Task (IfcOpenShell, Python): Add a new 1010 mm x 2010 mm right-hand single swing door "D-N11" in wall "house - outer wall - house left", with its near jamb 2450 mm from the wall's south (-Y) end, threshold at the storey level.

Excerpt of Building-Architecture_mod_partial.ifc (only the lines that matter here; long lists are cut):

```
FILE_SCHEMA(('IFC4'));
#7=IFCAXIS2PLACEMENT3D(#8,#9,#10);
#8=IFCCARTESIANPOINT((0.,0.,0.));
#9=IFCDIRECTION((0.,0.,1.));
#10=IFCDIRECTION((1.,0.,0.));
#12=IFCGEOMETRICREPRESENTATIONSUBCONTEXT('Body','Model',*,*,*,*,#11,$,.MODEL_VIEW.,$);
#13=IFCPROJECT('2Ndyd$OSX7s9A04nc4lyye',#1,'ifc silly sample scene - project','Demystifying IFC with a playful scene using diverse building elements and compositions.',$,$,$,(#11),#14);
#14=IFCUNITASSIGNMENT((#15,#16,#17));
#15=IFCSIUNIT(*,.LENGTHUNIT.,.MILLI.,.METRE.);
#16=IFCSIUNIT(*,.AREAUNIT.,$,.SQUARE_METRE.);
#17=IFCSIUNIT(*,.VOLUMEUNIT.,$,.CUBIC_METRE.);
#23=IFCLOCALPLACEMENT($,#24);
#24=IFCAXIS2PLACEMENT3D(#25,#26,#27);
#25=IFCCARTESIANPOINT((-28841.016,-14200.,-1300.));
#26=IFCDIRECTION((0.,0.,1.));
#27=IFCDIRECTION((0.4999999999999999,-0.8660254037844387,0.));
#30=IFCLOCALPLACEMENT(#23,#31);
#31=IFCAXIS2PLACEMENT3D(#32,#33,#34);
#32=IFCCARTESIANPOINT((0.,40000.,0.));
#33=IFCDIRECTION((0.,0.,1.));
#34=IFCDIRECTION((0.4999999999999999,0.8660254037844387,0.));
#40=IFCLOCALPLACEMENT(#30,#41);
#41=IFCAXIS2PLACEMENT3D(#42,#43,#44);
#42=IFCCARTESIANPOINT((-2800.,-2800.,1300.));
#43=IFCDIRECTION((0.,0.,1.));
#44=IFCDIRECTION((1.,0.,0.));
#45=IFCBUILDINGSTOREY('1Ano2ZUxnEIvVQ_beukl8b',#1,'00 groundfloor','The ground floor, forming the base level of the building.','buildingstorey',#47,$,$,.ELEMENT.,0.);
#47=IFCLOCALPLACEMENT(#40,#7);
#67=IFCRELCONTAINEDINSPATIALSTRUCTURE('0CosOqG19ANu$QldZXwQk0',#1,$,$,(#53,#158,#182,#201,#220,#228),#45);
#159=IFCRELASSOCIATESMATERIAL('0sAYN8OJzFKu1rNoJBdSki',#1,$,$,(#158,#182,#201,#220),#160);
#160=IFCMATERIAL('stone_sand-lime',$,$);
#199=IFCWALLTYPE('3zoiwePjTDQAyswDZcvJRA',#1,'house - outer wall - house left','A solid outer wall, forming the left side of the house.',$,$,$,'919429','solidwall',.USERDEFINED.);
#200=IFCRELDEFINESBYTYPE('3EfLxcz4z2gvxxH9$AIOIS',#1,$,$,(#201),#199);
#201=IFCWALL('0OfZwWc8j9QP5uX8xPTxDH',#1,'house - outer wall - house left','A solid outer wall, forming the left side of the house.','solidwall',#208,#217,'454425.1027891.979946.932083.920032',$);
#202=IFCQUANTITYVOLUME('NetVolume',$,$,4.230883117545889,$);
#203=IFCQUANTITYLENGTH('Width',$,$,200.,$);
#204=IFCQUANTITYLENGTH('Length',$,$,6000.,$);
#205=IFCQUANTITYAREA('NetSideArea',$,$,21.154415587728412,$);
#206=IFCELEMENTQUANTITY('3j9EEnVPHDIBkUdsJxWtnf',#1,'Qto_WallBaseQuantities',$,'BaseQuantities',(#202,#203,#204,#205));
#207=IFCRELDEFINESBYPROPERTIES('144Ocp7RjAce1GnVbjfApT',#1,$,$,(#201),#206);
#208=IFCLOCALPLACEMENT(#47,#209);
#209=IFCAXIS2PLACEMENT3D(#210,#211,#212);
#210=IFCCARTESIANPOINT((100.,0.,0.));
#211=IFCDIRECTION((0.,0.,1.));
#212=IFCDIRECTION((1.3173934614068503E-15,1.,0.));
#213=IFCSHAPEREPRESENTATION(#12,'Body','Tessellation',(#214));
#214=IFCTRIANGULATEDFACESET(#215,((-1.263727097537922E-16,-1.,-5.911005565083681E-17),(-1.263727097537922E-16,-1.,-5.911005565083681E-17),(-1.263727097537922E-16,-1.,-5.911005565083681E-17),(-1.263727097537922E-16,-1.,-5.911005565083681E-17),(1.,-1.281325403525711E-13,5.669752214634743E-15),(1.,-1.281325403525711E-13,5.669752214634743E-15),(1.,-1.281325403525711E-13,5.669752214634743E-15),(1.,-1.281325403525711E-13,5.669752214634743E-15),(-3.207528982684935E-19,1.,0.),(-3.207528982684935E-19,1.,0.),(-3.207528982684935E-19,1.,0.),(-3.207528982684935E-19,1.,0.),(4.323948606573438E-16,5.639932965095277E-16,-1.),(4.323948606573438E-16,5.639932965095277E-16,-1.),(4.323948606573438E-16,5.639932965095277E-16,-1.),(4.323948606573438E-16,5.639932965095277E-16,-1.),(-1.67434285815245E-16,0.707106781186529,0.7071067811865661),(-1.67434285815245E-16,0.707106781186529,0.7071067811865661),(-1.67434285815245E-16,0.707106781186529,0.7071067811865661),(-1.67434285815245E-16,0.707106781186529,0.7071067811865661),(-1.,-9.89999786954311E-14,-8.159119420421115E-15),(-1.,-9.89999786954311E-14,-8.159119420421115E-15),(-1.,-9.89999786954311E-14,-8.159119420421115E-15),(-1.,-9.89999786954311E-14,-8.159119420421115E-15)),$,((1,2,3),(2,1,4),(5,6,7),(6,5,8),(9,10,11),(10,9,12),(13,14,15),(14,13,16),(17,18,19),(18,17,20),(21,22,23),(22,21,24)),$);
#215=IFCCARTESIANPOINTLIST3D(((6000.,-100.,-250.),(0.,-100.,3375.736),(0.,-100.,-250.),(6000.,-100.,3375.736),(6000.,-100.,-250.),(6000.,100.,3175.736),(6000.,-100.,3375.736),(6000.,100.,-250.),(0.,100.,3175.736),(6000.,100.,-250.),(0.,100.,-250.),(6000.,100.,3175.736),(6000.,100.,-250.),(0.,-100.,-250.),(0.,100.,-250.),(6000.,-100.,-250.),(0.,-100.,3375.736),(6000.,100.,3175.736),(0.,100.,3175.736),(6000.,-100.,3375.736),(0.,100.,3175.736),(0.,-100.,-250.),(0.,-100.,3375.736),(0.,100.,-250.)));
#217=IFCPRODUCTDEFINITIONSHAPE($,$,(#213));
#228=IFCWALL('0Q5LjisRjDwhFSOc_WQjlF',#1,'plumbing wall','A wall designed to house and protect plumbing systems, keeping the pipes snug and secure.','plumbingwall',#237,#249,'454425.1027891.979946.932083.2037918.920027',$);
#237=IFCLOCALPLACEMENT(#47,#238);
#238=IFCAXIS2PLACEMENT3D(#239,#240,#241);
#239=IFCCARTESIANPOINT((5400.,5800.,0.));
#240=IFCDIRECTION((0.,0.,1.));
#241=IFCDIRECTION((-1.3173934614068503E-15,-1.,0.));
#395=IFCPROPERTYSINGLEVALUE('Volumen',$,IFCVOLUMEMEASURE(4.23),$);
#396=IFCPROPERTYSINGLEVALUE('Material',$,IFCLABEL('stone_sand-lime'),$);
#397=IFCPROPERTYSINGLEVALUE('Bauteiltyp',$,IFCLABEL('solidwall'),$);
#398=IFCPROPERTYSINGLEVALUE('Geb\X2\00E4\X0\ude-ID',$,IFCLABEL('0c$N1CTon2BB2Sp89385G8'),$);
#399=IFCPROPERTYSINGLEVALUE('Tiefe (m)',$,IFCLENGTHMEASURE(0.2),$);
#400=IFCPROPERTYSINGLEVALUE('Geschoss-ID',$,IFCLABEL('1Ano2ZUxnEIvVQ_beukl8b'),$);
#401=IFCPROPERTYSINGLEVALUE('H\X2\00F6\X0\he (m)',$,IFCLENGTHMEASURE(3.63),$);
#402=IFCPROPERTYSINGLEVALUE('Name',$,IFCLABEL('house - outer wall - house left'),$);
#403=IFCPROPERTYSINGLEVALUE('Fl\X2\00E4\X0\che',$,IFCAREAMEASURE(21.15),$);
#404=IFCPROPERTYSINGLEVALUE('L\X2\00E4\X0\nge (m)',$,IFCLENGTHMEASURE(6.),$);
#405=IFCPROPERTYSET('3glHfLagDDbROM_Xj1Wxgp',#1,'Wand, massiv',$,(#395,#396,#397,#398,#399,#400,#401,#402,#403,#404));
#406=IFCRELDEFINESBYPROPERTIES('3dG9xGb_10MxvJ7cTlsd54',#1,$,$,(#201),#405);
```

```python
import numpy as np
import ifcopenshell
import ifcopenshell.api.feature
import ifcopenshell.api.geometry
import ifcopenshell.api.pset
import ifcopenshell.api.root
import ifcopenshell.api.spatial
import ifcopenshell.geom
import ifcopenshell.util.element
import ifcopenshell.util.placement
import ifcopenshell.util.representation
import ifcopenshell.util.shape
import ifcopenshell.util.unit

model = ifcopenshell.open("Building-Architecture_mod_partial.ifc")
unit_scale = ifcopenshell.util.unit.calculate_unit_scale(model)
area_scale = ifcopenshell.util.unit.calculate_unit_scale(model, "AREAUNIT")
volume_scale = ifcopenshell.util.unit.calculate_unit_scale(model, "VOLUMEUNIT")
settings = ifcopenshell.geom.settings()


def volume(element):
    """Net volume in cubic metres, openings subtracted."""
    shape = ifcopenshell.geom.create_shape(settings, element)
    return ifcopenshell.util.shape.get_volume(shape.geometry)


wall = model.by_guid("0OfZwWc8j9QP5uX8xPTxDH")
storey = ifcopenshell.util.element.get_container(wall, ifc_class="IfcBuildingStorey")
context = ifcopenshell.util.representation.get_context(model, "Model", "Body", "MODEL_VIEW")
before = volume(wall)

width, height, from_end, sill = 1.01, 2.01, 2.45, 0.0  # metres

# The wall runs along its own X axis, and the end named is its -X end.
wall_shape = ifcopenshell.geom.create_shape(settings, wall)
x, y, z = ifcopenshell.util.shape.get_vertices(wall_shape.geometry).T
start = x.min() + from_end
face, thickness = float(y.min()), float(y.max() - y.min())
wall_matrix = ifcopenshell.util.placement.get_local_placement(wall.ObjectPlacement)
level = ifcopenshell.util.placement.get_local_placement(storey.ObjectPlacement)[2, 3]


def in_wall(x, y):
    """Placement at x, y metres in the wall's axes, at sill height."""
    matrix = wall_matrix.copy()
    matrix[:, 3] = wall_matrix @ np.array([x / unit_scale, y / unit_scale, 0.0, 1.0])
    matrix[2, 3] = level + sill / unit_scale
    return matrix


# Opening: a box that overshoots both wall faces by 50 mm.
opening = ifcopenshell.api.root.create_entity(model, ifc_class="IfcOpeningElement", predefined_type="OPENING")
box = ifcopenshell.api.geometry.add_wall_representation(
    model, context=context, length=width, height=height, thickness=thickness + 0.1
)
ifcopenshell.api.geometry.assign_representation(model, product=opening, representation=box)
ifcopenshell.api.geometry.edit_object_placement(model, product=opening, matrix=in_wall(start, face - 0.05), is_si=False)
ifcopenshell.api.feature.add_feature(model, feature=opening, element=wall)

door = ifcopenshell.api.root.create_entity(model, ifc_class="IfcDoor", name="D-N11", predefined_type="DOOR")
door.OverallWidth, door.OverallHeight = width / unit_scale, height / unit_scale
door.OperationType = "SINGLE_SWING_RIGHT"
body = ifcopenshell.api.geometry.add_door_representation(
    model,
    context=context,
    overall_width=door.OverallWidth,
    overall_height=door.OverallHeight,
    operation_type="SINGLE_SWING_RIGHT",
    lining_properties={"LiningDepth": thickness / unit_scale, "ThresholdDepth": thickness / unit_scale},
)
ifcopenshell.api.geometry.assign_representation(model, product=door, representation=body)
ifcopenshell.api.spatial.assign_container(model, products=[door], relating_structure=storey)
ifcopenshell.api.feature.add_filling(model, opening=opening, element=door)

# The lining spans the wall, so the door starts at the wall face.
ifcopenshell.api.geometry.edit_object_placement(model, product=door, matrix=in_wall(start, face), is_si=False)

after = volume(wall)

# Update the wall's stored quantities.
qto = model.by_id(ifcopenshell.util.element.get_pset(wall, "Qto_WallBaseQuantities", should_inherit=False)["id"])
ifcopenshell.api.pset.edit_qto(model, qto=qto, properties={
    "NetVolume": after / volume_scale,
    "NetSideArea": after / thickness / area_scale,
})
pset = model.by_id(ifcopenshell.util.element.get_pset(wall, "Wand, massiv", should_inherit=False)["id"])
ifcopenshell.api.pset.edit_pset(model, pset=pset, properties={
    "Volumen": model.create_entity("IfcVolumeMeasure", after / volume_scale),
    "Fläche": model.create_entity("IfcAreaMeasure", after / thickness / area_scale),
})

print(f"wall volume {before:.3f} -> {after:.3f} m3")

model.write("Building-Architecture_mod_partial_edited.ifc")
```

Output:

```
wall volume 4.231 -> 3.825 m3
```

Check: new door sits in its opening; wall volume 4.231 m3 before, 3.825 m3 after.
